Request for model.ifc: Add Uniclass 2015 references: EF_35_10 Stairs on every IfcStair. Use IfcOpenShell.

First a look at what the model holds.

```python
import ifcopenshell

model = ifcopenshell.open("model.ifc")
print(model.schema)
print("classifications:", [c.Name for c in model.by_type("IfcClassification")])
for ifc_class in ("IfcDoor", "IfcRoof", "IfcStair", "IfcWall", "IfcWindow"):
    print(ifc_class, len(model.by_type(ifc_class)))
```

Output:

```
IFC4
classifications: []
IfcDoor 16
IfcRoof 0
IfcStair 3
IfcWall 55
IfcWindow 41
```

```python
import ifcopenshell
import ifcopenshell.api.classification

model = ifcopenshell.open("model.ifc")

system = ifcopenshell.api.classification.add_classification(model, classification="Uniclass 2015")

codes = {
    "IfcStair": ("EF_35_10", "Stairs"),
}
for ifc_class, (code, name) in codes.items():
    products = model.by_type(ifc_class)
    ifcopenshell.api.classification.add_reference(
        model, products=products, classification=system, identification=code, name=name
    )
    print(code, len(products))

model.write("model_updated.ifc")
```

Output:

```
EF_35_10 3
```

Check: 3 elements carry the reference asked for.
